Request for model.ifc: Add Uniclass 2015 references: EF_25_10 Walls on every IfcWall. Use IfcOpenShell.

First a look at what the model holds.

```python
import ifcopenshell

model = ifcopenshell.open("model.ifc")
print(model.schema)
print("classifications:", [c.Name for c in model.by_type("IfcClassification")])
for ifc_class in ("IfcDoor", "IfcRoof", "IfcStair", "IfcWall", "IfcWindow"):
    print(ifc_class, len(model.by_type(ifc_class)))
```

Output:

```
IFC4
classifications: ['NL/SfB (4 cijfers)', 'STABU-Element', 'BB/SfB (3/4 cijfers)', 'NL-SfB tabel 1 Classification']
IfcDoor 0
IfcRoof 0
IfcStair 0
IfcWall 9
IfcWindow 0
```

```python
import ifcopenshell
import ifcopenshell.api.classification

model = ifcopenshell.open("model.ifc")

system = ifcopenshell.api.classification.add_classification(model, classification="Uniclass 2015")

codes = {
    "IfcWall": ("EF_25_10", "Walls"),
}
for ifc_class, (code, name) in codes.items():
    products = model.by_type(ifc_class)
    ifcopenshell.api.classification.add_reference(
        model, products=products, classification=system, identification=code, name=name
    )
    print(code, len(products))

model.write("model_v2.ifc")
```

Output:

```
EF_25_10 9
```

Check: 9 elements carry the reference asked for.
